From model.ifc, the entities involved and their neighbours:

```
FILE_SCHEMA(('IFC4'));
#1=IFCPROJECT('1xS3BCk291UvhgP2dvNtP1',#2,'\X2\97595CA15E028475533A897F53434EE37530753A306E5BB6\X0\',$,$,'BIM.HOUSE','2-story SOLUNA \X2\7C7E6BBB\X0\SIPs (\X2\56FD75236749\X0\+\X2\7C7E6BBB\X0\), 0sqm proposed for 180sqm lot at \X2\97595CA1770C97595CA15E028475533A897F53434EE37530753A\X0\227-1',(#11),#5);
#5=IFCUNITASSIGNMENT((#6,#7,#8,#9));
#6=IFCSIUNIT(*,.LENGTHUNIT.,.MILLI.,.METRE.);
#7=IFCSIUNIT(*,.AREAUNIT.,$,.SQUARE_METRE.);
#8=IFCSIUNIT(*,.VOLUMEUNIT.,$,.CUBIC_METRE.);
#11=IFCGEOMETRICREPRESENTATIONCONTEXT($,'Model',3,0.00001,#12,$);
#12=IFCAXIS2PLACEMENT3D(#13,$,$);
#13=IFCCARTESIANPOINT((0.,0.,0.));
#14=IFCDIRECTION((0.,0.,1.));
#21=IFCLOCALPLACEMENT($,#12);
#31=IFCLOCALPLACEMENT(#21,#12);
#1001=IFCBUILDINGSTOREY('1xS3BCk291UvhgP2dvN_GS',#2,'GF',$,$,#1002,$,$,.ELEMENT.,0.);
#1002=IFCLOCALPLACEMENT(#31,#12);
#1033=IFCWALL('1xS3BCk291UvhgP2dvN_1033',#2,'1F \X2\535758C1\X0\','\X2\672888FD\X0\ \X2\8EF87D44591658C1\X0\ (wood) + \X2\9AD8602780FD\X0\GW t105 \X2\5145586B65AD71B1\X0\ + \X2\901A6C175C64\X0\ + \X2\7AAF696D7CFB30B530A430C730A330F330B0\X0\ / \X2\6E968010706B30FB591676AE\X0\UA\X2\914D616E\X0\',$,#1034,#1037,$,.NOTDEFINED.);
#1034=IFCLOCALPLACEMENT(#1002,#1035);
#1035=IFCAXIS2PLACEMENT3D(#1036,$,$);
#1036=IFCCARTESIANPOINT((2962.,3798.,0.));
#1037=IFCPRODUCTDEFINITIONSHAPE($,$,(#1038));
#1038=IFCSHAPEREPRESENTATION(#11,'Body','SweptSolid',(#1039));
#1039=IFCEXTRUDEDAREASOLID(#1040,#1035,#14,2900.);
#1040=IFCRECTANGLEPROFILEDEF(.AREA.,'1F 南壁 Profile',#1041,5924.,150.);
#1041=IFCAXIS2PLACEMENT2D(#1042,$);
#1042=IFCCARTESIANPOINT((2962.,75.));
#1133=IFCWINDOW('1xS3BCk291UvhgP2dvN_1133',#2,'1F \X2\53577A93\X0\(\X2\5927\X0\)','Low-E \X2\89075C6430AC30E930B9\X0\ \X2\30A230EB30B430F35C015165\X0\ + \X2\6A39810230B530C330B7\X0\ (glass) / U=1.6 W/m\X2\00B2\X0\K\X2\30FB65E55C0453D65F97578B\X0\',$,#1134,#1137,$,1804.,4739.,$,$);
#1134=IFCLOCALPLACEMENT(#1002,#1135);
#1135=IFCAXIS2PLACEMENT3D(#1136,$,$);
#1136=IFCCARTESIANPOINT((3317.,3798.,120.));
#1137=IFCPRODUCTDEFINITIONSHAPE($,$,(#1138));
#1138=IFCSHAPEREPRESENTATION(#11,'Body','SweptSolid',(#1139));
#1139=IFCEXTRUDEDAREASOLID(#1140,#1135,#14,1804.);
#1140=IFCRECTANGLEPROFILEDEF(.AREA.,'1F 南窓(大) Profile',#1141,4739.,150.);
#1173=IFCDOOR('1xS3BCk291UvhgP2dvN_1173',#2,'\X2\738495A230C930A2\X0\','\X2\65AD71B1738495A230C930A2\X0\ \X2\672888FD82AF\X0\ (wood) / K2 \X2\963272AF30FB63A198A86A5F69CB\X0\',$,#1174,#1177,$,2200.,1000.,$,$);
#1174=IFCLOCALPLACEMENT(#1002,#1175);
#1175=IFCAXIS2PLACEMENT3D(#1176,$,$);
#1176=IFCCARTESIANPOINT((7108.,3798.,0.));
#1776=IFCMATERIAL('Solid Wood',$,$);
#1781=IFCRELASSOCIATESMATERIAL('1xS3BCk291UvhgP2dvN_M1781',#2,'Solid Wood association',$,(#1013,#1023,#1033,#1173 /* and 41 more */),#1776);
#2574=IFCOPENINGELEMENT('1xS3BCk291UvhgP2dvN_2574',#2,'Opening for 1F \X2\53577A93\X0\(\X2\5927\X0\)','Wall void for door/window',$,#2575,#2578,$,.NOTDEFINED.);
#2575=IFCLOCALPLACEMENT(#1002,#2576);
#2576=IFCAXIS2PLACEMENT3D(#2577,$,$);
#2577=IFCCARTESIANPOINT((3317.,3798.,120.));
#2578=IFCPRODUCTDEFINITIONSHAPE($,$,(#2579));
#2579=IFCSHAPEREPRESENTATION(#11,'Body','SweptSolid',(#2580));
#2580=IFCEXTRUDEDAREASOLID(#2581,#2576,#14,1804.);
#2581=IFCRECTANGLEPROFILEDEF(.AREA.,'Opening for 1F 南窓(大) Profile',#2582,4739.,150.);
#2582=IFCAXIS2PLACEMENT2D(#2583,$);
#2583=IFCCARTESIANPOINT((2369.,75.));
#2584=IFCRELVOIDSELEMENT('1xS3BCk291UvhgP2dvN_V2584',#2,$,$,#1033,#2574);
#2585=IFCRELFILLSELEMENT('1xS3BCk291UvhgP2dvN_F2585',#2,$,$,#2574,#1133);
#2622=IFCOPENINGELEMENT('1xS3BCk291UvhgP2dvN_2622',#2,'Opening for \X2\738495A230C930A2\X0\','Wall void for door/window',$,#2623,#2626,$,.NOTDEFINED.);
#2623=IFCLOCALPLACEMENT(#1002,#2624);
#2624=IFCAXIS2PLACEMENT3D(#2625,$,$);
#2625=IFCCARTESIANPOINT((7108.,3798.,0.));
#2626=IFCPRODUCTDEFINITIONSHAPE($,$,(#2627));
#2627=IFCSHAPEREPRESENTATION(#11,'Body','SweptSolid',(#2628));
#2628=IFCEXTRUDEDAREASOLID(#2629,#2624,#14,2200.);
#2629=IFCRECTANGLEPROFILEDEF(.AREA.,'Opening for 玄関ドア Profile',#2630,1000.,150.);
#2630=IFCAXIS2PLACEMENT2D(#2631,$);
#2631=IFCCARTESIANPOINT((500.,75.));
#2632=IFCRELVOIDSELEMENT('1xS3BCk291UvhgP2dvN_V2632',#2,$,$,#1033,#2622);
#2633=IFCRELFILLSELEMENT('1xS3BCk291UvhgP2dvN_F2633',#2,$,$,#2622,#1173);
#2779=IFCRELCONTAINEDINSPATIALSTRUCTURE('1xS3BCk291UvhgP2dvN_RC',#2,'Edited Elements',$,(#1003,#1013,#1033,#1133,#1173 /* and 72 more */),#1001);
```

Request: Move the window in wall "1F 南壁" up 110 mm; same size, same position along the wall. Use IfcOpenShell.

```python
import numpy as np
import ifcopenshell
import ifcopenshell.api.geometry
import ifcopenshell.util.placement
import ifcopenshell.util.unit

model = ifcopenshell.open("model.ifc")
unit_scale = ifcopenshell.util.unit.calculate_unit_scale(model)

window = model.by_id(1133)
opening = window.FillsVoids[0].RelatingOpeningElement
dz = 110.0

shift = np.array([0.0, 0.0, dz])
# The window is not placed relative to its opening, so move both.
for product in (opening, window):
    matrix = ifcopenshell.util.placement.get_local_placement(product.ObjectPlacement)
    matrix[:3, 3] += shift
    ifcopenshell.api.geometry.edit_object_placement(model, product=product, matrix=matrix, is_si=False)

print(f"moved by {dz * unit_scale:+.3f} m")

model.write("model_v2.ifc")
```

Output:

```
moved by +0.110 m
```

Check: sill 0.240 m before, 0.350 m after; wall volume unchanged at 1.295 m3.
